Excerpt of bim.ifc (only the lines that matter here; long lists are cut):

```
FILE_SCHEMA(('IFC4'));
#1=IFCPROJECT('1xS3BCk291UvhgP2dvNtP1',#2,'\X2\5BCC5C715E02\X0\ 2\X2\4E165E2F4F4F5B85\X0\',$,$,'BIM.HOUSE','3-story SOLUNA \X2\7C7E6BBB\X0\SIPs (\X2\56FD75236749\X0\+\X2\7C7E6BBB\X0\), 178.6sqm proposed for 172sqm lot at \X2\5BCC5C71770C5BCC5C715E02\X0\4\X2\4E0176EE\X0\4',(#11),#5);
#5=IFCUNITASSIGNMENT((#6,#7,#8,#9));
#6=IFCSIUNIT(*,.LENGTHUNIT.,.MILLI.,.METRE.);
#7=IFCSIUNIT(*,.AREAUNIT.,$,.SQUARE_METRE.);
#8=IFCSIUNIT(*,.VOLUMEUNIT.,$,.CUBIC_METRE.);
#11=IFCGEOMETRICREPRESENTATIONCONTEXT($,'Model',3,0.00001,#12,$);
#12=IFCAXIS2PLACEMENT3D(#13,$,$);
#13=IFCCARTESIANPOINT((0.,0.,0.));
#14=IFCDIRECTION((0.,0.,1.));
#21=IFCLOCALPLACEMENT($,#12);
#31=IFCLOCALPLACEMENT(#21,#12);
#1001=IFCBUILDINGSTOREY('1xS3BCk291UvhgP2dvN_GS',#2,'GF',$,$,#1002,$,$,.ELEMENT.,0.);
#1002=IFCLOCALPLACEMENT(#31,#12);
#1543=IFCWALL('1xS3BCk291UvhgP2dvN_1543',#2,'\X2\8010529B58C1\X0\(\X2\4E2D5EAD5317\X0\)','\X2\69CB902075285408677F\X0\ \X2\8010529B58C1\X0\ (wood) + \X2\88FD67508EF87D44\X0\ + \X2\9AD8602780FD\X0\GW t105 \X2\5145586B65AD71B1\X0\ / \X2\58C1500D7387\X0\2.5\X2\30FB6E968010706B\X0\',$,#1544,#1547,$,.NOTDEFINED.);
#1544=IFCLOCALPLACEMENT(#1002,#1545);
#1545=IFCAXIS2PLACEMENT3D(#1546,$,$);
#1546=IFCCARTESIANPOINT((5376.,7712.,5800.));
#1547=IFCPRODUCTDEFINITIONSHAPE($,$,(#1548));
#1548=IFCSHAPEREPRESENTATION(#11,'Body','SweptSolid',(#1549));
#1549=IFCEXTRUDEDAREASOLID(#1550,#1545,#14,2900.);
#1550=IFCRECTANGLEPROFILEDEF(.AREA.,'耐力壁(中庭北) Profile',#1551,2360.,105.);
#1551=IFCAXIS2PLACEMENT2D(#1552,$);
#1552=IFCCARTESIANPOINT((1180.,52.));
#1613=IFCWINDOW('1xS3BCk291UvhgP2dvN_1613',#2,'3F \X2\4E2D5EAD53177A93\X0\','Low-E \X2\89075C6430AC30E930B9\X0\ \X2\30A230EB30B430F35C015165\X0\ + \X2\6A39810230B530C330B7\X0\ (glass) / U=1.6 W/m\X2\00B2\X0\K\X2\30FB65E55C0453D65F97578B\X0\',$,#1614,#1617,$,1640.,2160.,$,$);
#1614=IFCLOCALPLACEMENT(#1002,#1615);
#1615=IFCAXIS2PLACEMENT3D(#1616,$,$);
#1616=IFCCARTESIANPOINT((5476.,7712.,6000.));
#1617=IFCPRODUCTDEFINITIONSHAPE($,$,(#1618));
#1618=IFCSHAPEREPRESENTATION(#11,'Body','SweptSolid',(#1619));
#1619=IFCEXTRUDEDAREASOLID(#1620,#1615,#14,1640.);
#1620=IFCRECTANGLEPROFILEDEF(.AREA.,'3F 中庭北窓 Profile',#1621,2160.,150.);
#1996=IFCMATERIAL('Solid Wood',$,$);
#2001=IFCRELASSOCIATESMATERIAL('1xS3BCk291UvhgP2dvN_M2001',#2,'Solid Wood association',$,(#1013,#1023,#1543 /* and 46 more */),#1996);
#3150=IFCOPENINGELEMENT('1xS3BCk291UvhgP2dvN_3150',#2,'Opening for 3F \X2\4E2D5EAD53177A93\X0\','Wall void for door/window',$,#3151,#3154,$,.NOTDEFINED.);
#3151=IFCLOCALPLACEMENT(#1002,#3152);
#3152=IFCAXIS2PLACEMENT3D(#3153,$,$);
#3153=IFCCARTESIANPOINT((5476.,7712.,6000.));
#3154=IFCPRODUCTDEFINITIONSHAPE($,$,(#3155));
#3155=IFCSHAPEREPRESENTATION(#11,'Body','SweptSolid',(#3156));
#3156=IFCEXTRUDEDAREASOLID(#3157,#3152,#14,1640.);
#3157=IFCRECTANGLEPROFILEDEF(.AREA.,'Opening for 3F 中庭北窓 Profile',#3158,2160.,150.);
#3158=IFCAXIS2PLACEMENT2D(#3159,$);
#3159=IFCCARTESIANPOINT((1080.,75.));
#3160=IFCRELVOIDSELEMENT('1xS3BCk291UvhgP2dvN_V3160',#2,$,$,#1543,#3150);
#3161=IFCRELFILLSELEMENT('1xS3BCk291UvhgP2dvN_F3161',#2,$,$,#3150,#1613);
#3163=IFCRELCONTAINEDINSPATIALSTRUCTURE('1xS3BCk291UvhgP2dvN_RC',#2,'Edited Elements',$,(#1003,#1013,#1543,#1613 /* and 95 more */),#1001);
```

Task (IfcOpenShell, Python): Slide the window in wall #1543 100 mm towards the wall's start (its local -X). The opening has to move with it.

```python
import ifcopenshell
import ifcopenshell.api.geometry
import ifcopenshell.util.placement

model = ifcopenshell.open("bim.ifc")

window = model.by_id(1613)
opening = window.FillsVoids[0].RelatingOpeningElement
wall = opening.VoidsElements[0].RelatingBuildingElement

wall_matrix = ifcopenshell.util.placement.get_local_placement(wall.ObjectPlacement)
shift = wall_matrix[:3, 0] * -100.0
before = ifcopenshell.util.placement.get_local_placement(window.ObjectPlacement)[:3, 3].copy()

# The window is not placed relative to its opening, so move both.
for product in (opening, window):
    matrix = ifcopenshell.util.placement.get_local_placement(product.ObjectPlacement)
    matrix[:3, 3] += shift
    ifcopenshell.api.geometry.edit_object_placement(model, product=product, matrix=matrix, is_si=False)

after = ifcopenshell.util.placement.get_local_placement(window.ObjectPlacement)[:3, 3]
print("window moved by", (after - before).round(3) + 0.0)

model.write("bim_edited.ifc")
```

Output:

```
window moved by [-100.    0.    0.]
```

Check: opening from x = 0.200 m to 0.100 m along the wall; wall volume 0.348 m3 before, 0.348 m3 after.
